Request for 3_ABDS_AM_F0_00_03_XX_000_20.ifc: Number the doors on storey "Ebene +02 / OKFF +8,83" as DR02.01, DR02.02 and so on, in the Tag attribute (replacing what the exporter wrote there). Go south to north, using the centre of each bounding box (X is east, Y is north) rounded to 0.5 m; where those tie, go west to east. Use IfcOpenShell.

First a look at what the model holds.

```python
import ifcopenshell
import ifcopenshell.util.element
import ifcopenshell.util.placement

model = ifcopenshell.open("3_ABDS_AM_F0_00_03_XX_000_20.ifc")
print(model.schema)
storey = next(s for s in model.by_type("IfcBuildingStorey") if s.Name == "Ebene +02 / OKFF +8,83")
doors = [e for e in ifcopenshell.util.element.get_decomposition(storey) if e.is_a("IfcDoor")]
for e in sorted(doors, key=lambda e: e.id()):
    origin = ifcopenshell.util.placement.get_local_placement(e.ObjectPlacement)[:3, 3]
    print(e.id(), e.Tag, e.Name, origin.round(2) + 0.0, sep=" | ")
```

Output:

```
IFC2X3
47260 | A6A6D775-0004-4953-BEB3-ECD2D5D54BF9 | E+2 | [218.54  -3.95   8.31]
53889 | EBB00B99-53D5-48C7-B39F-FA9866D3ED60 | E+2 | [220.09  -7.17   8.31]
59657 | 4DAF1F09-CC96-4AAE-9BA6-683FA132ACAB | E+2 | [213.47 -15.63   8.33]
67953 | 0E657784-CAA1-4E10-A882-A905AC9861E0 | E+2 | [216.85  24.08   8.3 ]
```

```python
import ifcopenshell
import ifcopenshell.geom
import ifcopenshell.util.element
import ifcopenshell.util.shape

model = ifcopenshell.open("3_ABDS_AM_F0_00_03_XX_000_20.ifc")
settings = ifcopenshell.geom.settings()
settings.set("use-world-coords", True)


def centre(element):
    shape = ifcopenshell.geom.create_shape(settings, element)
    return ifcopenshell.util.shape.get_bbox_centroid(shape.geometry)


storey = next(s for s in model.by_type("IfcBuildingStorey") if s.Name == "Ebene +02 / OKFF +8,83")
doors = [e for e in ifcopenshell.util.element.get_decomposition(storey) if e.is_a("IfcDoor")]

# Insertion points can sit at a corner or the storey origin, so sort by the geometry (in metres).
centres = {e: centre(e) for e in doors}
doors.sort(key=lambda e: (round(centres[e][1] / 0.5), centres[e][0]))

for i, e in enumerate(doors, start=1):
    number = f"DR02.{i:02d}"
    e.Tag = number
    print(e.id(), number)

model.write("3_ABDS_AM_F0_00_03_XX_000_20_edited.ifc")
```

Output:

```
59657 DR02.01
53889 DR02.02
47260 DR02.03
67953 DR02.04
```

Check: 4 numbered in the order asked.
